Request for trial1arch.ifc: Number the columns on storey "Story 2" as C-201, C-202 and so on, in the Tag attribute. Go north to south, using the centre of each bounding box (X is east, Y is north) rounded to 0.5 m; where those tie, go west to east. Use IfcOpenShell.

First a look at what the model holds.

```python
import ifcopenshell
import ifcopenshell.util.element
import ifcopenshell.util.placement

model = ifcopenshell.open("trial1arch.ifc")
print(model.schema)
storey = next(s for s in model.by_type("IfcBuildingStorey") if s.Name == "Story 2")
columns = [e for e in ifcopenshell.util.element.get_decomposition(storey) if e.is_a("IfcColumn")]
for e in sorted(columns, key=lambda e: e.id()):
    origin = ifcopenshell.util.placement.get_local_placement(e.ObjectPlacement)[:3, 3]
    print(e.id(), e.Tag, e.Name, origin.round(2) + 0.0, sep=" | ")
```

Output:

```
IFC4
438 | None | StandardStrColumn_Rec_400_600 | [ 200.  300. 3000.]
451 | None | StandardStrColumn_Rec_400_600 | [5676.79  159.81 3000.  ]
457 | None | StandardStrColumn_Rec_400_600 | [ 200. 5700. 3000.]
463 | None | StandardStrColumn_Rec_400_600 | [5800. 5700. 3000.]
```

```python
import ifcopenshell
import ifcopenshell.geom
import ifcopenshell.util.element
import ifcopenshell.util.shape

model = ifcopenshell.open("trial1arch.ifc")
settings = ifcopenshell.geom.settings()
settings.set("use-world-coords", True)


def centre(element):
    shape = ifcopenshell.geom.create_shape(settings, element)
    return ifcopenshell.util.shape.get_bbox_centroid(shape.geometry)


storey = next(s for s in model.by_type("IfcBuildingStorey") if s.Name == "Story 2")
columns = [e for e in ifcopenshell.util.element.get_decomposition(storey) if e.is_a("IfcColumn")]

# Insertion points can sit at a corner or the storey origin, so sort by the geometry (in metres).
centres = {e: centre(e) for e in columns}
columns.sort(key=lambda e: (-round(centres[e][1] / 0.5), centres[e][0]))

for i, e in enumerate(columns, start=1):
    number = f"C-2{i:02d}"
    e.Tag = number
    print(e.id(), number)

model.write("trial1arch_v2.ifc")
```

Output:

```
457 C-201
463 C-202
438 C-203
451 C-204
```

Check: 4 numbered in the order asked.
